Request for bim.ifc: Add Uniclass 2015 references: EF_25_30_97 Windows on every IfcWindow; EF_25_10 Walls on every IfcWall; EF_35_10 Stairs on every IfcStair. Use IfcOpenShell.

First a look at what the model holds.

```python
import ifcopenshell

model = ifcopenshell.open("bim.ifc")
print(model.schema)
print("classifications:", [c.Name for c in model.by_type("IfcClassification")])
for ifc_class in ("IfcDoor", "IfcRoof", "IfcStair", "IfcWall", "IfcWindow"):
    print(ifc_class, len(model.by_type(ifc_class)))
```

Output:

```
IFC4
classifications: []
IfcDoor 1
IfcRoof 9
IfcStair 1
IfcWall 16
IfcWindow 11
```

```python
import ifcopenshell
import ifcopenshell.api.classification

model = ifcopenshell.open("bim.ifc")

system = ifcopenshell.api.classification.add_classification(model, classification="Uniclass 2015")

codes = {
    "IfcWindow": ("EF_25_30_97", "Windows"),
    "IfcWall": ("EF_25_10", "Walls"),
    "IfcStair": ("EF_35_10", "Stairs"),
}
for ifc_class, (code, name) in codes.items():
    products = model.by_type(ifc_class)
    ifcopenshell.api.classification.add_reference(
        model, products=products, classification=system, identification=code, name=name
    )
    print(code, len(products))

model.write("bim-out.ifc")
```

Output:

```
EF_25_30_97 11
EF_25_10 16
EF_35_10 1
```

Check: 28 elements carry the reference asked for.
